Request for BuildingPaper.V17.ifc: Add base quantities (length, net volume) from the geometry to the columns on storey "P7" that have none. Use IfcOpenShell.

First a look at what the model holds.

```python
import ifcopenshell
import ifcopenshell.util.element
import ifcopenshell.util.unit

model = ifcopenshell.open("BuildingPaper.V17.ifc")
print(model.schema)
for unit_type in ("LENGTHUNIT", "AREAUNIT", "VOLUMEUNIT"):
    print(unit_type, ifcopenshell.util.unit.calculate_unit_scale(model, unit_type))
storey = next(s for s in model.by_type("IfcBuildingStorey") if s.Name == "P7")
columns = [e for e in ifcopenshell.util.element.get_decomposition(storey) if e.is_a("IfcColumn")]
for e in sorted(columns, key=lambda e: e.id()):
    print(e.id(), e.is_a(), e.Name, list(ifcopenshell.util.element.get_psets(e, qtos_only=True)), sep=" | ")
```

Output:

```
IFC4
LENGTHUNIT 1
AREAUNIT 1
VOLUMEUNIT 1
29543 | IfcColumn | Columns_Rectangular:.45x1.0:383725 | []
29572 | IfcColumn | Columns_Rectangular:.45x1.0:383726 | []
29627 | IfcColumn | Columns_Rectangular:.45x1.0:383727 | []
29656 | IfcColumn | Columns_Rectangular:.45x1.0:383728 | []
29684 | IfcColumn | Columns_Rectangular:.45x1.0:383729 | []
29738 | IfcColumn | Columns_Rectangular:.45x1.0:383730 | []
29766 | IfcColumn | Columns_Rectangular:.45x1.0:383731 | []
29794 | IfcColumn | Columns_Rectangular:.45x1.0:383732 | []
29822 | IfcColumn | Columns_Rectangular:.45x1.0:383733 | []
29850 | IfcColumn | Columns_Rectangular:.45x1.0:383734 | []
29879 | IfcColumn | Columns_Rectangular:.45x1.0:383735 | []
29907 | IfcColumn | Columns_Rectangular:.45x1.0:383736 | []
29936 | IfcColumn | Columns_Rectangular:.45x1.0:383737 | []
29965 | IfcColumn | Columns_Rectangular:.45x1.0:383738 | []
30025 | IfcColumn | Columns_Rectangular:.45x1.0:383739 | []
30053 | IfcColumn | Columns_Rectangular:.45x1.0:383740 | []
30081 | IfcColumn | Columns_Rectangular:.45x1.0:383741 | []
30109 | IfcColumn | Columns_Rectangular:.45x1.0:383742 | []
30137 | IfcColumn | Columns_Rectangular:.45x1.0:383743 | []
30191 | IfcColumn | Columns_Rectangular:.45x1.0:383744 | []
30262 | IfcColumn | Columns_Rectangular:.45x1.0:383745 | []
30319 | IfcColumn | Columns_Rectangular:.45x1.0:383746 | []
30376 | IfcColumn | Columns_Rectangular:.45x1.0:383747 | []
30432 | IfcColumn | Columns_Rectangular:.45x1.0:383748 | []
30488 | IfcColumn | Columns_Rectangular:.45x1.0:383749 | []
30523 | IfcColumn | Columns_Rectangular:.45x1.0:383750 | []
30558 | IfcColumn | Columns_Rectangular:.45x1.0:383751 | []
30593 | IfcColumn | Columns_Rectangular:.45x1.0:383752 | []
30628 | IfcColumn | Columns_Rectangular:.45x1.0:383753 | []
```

```python
import ifcopenshell
import ifcopenshell.api.pset
import ifcopenshell.geom
import ifcopenshell.util.element
import ifcopenshell.util.shape
import ifcopenshell.util.unit

model = ifcopenshell.open("BuildingPaper.V17.ifc")
unit_scale = ifcopenshell.util.unit.calculate_unit_scale(model)
volume_scale = ifcopenshell.util.unit.calculate_unit_scale(model, "VOLUMEUNIT")
settings = ifcopenshell.geom.settings()

storey = next(s for s in model.by_type("IfcBuildingStorey") if s.Name == "P7")
columns = [e for e in ifcopenshell.util.element.get_decomposition(storey) if e.is_a("IfcColumn")]

for e in sorted(columns, key=lambda e: e.id()):
    if ifcopenshell.util.element.get_psets(e, qtos_only=True, should_inherit=False):
        continue
    # Geometry comes back in metres, in the element's own axes.
    shape = ifcopenshell.geom.create_shape(settings, e)
    values = {
        "Length": ifcopenshell.util.shape.get_z(shape.geometry) / unit_scale,
        "NetVolume": ifcopenshell.util.shape.get_volume(shape.geometry) / volume_scale,
    }
    qto = ifcopenshell.api.pset.add_qto(model, product=e, name="Qto_ColumnBaseQuantities")
    ifcopenshell.api.pset.edit_qto(model, qto=qto, properties=values)
    print(e.id(), {k: round(v, 3) for k, v in values.items()})

model.write("BuildingPaper.V17_v2.ifc")
```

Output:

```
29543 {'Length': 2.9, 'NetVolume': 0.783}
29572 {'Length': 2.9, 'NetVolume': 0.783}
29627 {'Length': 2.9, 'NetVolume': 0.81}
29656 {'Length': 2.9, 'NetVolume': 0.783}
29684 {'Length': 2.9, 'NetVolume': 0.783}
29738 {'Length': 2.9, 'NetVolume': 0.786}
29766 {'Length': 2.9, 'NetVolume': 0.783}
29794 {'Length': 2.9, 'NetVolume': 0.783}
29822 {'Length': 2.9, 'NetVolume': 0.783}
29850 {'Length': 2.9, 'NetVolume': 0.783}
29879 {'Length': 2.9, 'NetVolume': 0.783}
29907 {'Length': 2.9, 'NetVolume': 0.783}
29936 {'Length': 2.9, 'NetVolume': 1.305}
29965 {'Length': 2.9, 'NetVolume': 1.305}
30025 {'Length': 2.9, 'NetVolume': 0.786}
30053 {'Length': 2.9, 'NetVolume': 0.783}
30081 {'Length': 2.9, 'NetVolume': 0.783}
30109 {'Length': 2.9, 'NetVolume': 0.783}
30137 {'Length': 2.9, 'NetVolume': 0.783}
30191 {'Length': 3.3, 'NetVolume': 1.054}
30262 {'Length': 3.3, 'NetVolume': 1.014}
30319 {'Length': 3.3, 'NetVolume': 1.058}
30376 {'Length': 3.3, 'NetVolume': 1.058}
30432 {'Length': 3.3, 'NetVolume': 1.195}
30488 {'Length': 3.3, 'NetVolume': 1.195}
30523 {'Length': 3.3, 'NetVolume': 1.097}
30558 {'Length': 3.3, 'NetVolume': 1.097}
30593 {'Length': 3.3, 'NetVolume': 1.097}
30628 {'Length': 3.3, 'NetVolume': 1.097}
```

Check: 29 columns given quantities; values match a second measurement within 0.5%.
